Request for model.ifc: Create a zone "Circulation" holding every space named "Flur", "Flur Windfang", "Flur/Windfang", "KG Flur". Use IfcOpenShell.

First a look at what the model holds.

```python
import ifcopenshell

model = ifcopenshell.open("model.ifc")
print(model.schema)
seen = {}
for space in model.by_type("IfcSpace"):
    seen[space.LongName] = seen.get(space.LongName, 0) + 1
for name, count in sorted(seen.items(), key=str):
    print(count, "x", name)
print("zones:", [z.Name for z in model.by_type("IfcZone")][:20])
```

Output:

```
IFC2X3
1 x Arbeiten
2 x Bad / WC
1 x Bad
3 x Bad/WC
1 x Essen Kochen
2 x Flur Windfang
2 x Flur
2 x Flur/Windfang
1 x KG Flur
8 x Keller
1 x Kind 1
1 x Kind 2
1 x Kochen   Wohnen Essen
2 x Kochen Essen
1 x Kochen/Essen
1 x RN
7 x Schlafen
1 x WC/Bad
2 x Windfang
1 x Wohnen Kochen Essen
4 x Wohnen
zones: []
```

```python
import ifcopenshell
import ifcopenshell.api.group
import ifcopenshell.api.root

model = ifcopenshell.open("model.ifc")

names = {"Flur", "Flur Windfang", "Flur/Windfang", "KG Flur"}
spaces = [s for s in model.by_type("IfcSpace") if s.LongName in names]

zone = ifcopenshell.api.root.create_entity(model, ifc_class="IfcZone", name="Circulation")
ifcopenshell.api.group.assign_group(model, products=spaces, group=zone)
print(len(spaces), "spaces in", zone.Name)

model.write("model_edited.ifc")
```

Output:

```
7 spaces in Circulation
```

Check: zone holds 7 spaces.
